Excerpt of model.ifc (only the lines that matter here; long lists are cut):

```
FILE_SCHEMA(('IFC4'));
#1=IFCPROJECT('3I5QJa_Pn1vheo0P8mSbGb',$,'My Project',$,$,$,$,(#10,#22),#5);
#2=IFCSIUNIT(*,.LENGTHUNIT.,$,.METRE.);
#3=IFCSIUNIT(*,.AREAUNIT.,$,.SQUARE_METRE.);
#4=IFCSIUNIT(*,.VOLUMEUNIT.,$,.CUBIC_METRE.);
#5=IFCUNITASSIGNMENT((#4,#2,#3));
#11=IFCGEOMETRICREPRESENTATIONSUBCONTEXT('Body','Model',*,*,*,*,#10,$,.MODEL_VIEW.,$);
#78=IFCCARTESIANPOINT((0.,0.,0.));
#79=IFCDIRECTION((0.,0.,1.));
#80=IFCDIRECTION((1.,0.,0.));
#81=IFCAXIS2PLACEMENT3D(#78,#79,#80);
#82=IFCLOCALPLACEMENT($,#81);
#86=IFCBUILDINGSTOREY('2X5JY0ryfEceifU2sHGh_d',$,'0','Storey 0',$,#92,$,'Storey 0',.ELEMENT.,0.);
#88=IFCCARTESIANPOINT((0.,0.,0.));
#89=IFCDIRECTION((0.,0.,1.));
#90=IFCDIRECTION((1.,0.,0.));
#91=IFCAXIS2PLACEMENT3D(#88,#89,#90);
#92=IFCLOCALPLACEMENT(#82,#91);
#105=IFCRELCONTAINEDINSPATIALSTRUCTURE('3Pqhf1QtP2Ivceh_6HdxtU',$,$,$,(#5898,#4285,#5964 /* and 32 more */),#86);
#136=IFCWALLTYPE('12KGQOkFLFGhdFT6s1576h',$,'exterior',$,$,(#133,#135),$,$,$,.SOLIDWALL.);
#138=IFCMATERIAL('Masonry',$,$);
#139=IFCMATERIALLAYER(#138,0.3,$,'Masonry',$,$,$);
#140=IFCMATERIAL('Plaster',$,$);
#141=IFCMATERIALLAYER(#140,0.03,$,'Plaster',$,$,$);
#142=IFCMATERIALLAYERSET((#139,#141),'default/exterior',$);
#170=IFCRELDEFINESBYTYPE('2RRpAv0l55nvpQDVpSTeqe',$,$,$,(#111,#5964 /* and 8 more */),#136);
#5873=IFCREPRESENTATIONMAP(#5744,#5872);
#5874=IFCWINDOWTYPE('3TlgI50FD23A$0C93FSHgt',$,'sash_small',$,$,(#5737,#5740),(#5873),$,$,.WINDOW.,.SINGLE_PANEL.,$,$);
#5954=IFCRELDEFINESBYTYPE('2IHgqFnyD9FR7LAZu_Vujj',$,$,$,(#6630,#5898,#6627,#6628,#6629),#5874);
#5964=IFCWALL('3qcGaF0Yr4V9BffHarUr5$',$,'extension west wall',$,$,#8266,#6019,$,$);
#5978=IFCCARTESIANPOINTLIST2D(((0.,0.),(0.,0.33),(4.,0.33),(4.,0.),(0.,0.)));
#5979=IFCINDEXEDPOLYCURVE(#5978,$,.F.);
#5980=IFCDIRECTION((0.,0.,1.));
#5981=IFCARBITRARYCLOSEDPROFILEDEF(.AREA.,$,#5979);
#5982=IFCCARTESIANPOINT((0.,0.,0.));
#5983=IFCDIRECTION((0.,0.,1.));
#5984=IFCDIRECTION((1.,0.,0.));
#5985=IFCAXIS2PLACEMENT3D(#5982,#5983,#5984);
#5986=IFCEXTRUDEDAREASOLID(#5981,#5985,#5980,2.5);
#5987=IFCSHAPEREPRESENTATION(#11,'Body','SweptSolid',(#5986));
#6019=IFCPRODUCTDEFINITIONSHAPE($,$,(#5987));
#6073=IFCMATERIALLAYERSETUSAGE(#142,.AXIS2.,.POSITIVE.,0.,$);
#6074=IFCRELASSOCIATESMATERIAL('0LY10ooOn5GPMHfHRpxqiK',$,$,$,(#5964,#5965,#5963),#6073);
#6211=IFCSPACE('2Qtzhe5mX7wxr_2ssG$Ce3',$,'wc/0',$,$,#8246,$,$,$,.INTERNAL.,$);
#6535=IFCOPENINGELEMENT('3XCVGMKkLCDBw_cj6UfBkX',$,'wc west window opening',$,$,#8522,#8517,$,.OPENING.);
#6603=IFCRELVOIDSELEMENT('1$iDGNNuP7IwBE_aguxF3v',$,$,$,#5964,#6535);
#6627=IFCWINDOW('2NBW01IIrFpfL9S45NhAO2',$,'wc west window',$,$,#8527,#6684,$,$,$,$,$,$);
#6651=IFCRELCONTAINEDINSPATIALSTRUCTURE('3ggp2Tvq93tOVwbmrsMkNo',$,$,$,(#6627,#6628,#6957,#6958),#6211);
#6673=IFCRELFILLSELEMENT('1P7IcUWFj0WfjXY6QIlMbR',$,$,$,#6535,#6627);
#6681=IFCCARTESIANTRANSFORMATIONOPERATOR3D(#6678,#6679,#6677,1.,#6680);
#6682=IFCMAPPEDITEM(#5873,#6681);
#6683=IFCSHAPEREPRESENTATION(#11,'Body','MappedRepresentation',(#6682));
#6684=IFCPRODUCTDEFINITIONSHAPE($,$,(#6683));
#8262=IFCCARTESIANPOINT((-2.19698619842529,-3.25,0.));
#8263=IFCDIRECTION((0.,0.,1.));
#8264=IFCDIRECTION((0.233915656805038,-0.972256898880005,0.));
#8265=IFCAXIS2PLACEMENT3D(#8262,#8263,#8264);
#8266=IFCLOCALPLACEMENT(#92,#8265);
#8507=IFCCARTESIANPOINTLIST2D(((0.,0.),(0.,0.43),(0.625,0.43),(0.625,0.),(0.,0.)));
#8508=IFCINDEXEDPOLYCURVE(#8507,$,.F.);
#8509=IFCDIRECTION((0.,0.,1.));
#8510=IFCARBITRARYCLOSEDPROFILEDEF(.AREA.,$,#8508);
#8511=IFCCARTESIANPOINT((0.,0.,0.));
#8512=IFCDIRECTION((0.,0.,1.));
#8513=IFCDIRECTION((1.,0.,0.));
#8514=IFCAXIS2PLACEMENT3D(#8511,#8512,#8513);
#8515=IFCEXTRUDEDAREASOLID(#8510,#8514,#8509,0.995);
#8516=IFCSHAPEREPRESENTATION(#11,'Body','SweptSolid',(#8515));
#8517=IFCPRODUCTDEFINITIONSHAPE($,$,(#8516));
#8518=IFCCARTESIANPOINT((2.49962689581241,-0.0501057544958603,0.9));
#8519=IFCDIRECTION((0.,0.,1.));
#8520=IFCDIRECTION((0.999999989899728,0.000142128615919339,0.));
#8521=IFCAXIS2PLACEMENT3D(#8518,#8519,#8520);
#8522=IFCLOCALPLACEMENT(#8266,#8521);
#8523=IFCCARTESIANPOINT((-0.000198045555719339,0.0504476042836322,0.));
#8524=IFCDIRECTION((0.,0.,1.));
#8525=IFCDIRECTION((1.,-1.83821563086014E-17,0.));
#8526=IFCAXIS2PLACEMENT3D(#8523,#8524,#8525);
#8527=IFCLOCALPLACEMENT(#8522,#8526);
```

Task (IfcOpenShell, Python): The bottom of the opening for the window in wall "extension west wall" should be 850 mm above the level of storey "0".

```python
import numpy as np
import ifcopenshell
import ifcopenshell.api.geometry
import ifcopenshell.geom
import ifcopenshell.util.element
import ifcopenshell.util.placement
import ifcopenshell.util.shape
import ifcopenshell.util.unit

model = ifcopenshell.open("model.ifc")
unit_scale = ifcopenshell.util.unit.calculate_unit_scale(model)

window = model.by_guid("2NBW01IIrFpfL9S45NhAO2")
opening = window.FillsVoids[0].RelatingOpeningElement
storey = ifcopenshell.util.element.get_container(window, ifc_class="IfcBuildingStorey")
level = ifcopenshell.util.placement.get_local_placement(storey.ObjectPlacement)[2, 3]

# The opening's origin need not be at the sill, so measure its lowest point.
shape = ifcopenshell.geom.create_shape(ifcopenshell.geom.settings(), opening)
bottom = ifcopenshell.util.shape.get_shape_bottom_elevation(shape, shape.geometry) / unit_scale
dz = level + 0.85 / unit_scale - bottom

shift = np.array([0.0, 0.0, dz])
# The window is placed relative to its opening, so it follows when the opening moves.
matrix = ifcopenshell.util.placement.get_local_placement(opening.ObjectPlacement)
matrix[:3, 3] += shift
ifcopenshell.api.geometry.edit_object_placement(
    model, product=opening, matrix=matrix, is_si=False, should_transform_children=True
)

print(f"moved by {dz * unit_scale:+.3f} m")

model.write("model_v2.ifc")
```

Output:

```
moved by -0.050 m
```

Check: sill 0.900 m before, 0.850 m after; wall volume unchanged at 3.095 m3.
